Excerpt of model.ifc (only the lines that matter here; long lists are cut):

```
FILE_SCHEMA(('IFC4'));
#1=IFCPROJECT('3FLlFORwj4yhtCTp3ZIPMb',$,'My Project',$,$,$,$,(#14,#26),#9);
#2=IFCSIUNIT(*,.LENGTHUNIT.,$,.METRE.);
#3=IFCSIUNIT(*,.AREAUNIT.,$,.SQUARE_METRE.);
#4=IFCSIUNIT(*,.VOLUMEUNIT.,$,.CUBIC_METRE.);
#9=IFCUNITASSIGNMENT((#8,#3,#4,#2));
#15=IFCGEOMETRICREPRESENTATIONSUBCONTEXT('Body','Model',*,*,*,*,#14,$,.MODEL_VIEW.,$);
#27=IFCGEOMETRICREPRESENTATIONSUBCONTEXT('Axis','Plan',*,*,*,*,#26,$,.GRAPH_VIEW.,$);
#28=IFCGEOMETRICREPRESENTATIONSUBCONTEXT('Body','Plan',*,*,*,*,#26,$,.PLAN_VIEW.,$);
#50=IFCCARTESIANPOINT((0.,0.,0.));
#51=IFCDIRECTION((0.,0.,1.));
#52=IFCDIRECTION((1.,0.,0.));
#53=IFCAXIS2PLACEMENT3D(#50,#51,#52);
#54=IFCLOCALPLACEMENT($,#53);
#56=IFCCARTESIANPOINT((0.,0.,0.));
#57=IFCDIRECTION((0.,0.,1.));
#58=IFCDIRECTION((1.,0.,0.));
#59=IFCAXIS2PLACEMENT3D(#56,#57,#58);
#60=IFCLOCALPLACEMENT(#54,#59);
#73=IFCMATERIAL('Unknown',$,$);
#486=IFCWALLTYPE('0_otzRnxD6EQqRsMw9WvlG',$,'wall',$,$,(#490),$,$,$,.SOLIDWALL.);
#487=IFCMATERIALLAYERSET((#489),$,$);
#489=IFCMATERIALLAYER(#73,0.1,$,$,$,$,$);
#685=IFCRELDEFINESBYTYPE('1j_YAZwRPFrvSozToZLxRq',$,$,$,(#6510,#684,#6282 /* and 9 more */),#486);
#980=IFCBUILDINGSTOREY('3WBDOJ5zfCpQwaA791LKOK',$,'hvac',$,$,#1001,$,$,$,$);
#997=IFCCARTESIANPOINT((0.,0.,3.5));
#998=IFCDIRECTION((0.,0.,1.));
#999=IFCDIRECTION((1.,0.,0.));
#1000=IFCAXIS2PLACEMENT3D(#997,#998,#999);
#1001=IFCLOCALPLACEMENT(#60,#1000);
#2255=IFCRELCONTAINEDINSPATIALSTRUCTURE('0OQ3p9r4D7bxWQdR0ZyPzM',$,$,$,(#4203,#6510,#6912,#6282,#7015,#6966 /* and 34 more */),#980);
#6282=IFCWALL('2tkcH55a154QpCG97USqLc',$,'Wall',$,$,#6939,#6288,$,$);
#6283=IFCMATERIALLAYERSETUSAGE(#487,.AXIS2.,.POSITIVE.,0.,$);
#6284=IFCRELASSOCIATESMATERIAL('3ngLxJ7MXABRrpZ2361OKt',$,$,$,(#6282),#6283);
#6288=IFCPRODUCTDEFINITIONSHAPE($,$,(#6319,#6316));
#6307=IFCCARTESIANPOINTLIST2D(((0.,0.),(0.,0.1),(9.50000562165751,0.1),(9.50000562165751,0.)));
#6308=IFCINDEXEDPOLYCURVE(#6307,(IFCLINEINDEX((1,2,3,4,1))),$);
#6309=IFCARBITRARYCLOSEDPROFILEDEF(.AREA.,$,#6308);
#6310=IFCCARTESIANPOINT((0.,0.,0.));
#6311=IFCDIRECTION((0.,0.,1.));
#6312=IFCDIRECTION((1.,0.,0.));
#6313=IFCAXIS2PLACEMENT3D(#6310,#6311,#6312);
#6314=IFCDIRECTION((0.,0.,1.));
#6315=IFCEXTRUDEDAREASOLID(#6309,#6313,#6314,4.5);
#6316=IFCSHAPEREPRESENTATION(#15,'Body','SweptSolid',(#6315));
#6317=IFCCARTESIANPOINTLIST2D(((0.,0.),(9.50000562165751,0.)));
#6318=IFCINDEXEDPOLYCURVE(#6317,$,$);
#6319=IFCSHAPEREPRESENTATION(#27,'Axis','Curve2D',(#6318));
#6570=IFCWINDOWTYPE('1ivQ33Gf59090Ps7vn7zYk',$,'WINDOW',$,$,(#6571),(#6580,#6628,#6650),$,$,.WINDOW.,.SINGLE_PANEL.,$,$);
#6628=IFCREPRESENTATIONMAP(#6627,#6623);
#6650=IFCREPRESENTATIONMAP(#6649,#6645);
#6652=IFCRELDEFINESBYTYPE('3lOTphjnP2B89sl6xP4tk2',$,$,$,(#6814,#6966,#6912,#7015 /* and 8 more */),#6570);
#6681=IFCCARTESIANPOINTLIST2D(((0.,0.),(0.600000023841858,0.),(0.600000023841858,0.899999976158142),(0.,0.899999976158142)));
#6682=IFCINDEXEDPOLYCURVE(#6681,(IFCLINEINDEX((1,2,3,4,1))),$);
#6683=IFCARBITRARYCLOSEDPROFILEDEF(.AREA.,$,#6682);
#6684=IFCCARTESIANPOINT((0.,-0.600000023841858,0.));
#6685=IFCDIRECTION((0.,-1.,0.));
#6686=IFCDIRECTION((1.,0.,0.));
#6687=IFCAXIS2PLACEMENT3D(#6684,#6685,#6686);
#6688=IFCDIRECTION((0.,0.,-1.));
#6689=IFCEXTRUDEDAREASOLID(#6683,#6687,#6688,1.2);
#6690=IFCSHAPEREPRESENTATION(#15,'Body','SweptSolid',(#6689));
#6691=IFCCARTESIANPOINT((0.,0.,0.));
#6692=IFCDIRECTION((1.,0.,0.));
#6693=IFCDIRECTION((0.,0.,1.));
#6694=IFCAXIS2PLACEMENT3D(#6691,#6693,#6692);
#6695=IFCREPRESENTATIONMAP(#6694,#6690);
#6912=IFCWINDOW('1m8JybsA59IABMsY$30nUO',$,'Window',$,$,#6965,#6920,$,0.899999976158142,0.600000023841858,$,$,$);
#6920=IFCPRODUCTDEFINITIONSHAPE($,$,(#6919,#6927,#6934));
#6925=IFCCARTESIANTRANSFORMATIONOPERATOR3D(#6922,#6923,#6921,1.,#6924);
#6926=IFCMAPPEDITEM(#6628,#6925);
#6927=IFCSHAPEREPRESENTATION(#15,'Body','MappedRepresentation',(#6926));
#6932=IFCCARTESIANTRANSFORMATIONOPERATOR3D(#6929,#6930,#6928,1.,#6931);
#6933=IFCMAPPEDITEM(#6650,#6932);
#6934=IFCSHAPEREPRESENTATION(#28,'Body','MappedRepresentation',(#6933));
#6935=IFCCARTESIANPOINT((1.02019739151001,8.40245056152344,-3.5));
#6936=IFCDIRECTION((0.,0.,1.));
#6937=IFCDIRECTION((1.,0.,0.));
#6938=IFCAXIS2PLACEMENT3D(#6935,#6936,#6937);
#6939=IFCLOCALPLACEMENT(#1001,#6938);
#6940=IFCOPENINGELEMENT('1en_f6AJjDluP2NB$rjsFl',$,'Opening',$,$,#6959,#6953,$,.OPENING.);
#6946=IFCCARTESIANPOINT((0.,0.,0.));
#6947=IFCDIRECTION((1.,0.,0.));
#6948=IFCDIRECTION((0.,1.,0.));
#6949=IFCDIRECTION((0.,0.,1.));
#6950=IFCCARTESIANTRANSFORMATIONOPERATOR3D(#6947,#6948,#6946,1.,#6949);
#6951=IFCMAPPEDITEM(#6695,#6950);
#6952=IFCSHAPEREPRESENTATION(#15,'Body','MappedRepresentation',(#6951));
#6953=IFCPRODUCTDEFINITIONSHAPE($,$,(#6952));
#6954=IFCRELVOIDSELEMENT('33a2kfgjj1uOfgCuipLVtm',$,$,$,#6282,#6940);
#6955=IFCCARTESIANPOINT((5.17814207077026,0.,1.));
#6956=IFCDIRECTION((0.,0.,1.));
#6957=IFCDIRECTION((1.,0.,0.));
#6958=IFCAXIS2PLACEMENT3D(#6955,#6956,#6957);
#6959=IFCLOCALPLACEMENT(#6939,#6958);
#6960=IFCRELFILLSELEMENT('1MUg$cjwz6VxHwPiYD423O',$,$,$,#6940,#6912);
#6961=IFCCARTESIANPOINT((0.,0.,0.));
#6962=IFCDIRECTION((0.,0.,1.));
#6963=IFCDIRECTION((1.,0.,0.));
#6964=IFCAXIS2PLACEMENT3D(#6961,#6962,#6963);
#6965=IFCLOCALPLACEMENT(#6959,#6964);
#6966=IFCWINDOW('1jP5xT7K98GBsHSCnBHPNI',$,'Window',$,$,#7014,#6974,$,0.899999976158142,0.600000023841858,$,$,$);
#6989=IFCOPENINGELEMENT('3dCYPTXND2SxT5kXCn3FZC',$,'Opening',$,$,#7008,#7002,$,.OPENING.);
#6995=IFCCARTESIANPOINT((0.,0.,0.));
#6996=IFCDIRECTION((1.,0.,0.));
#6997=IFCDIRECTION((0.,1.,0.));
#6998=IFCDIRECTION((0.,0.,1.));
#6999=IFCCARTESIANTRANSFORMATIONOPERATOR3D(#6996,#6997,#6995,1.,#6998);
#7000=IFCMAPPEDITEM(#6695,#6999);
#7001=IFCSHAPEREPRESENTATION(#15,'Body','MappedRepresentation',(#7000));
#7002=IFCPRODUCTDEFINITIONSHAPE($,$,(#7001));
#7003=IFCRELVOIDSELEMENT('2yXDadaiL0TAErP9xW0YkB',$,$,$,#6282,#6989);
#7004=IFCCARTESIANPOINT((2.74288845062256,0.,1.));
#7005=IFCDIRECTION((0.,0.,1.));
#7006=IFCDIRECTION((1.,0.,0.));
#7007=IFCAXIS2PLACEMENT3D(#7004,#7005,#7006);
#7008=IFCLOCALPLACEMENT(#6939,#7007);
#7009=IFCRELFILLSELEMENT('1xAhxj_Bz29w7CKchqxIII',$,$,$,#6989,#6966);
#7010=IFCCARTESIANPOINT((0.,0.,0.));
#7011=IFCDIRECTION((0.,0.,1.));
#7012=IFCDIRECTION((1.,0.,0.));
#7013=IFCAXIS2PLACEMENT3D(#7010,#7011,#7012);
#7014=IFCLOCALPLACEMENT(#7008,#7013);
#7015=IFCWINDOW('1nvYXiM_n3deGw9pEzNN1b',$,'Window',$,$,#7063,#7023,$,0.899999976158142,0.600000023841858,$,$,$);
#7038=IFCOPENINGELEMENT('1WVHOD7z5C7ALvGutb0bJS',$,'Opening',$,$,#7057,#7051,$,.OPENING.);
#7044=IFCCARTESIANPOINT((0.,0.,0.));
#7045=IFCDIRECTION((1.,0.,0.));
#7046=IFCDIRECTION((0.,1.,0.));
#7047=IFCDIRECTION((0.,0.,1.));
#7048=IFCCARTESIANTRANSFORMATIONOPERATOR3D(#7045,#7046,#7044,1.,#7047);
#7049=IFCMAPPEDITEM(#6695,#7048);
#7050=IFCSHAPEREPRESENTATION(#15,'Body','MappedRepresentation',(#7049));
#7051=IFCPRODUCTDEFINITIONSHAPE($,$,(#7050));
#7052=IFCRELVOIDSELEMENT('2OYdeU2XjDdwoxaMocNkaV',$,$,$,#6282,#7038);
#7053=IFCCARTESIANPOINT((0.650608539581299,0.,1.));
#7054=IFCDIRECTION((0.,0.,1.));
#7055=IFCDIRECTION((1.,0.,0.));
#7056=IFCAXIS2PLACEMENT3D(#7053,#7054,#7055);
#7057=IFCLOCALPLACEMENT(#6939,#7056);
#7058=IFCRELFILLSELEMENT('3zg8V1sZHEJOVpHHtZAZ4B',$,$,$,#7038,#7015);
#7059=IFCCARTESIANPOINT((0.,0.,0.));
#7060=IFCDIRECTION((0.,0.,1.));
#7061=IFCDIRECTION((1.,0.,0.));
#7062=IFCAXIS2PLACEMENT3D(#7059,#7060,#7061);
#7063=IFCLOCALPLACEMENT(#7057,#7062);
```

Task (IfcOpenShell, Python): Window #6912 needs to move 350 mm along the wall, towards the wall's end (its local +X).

```python
import ifcopenshell
import ifcopenshell.api.geometry
import ifcopenshell.util.placement
import ifcopenshell.util.unit

model = ifcopenshell.open("model.ifc")
unit_scale = ifcopenshell.util.unit.calculate_unit_scale(model)

window = model.by_guid("1m8JybsA59IABMsY$30nUO")
opening = window.FillsVoids[0].RelatingOpeningElement
wall = opening.VoidsElements[0].RelatingBuildingElement

wall_matrix = ifcopenshell.util.placement.get_local_placement(wall.ObjectPlacement)
shift = wall_matrix[:3, 0] * 0.35 / unit_scale
before = ifcopenshell.util.placement.get_local_placement(window.ObjectPlacement)[:3, 3].copy()

# The window is placed relative to its opening, so it follows when the opening moves.
matrix = ifcopenshell.util.placement.get_local_placement(opening.ObjectPlacement)
matrix[:3, 3] += shift
ifcopenshell.api.geometry.edit_object_placement(
    model, product=opening, matrix=matrix, is_si=False, should_transform_children=True
)

after = ifcopenshell.util.placement.get_local_placement(window.ObjectPlacement)[:3, 3]
print("window moved by", (after - before).round(3) + 0.0)

model.write("model_edited.ifc")
```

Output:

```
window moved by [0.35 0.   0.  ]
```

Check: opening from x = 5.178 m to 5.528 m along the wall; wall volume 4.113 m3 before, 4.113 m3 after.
